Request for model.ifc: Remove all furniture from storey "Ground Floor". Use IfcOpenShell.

First a look at what the model holds.

```python
import ifcopenshell
import ifcopenshell.util.element

model = ifcopenshell.open("model.ifc")
print(model.schema)
storey = next(s for s in model.by_type("IfcBuildingStorey") if s.Name == "Ground Floor")
furniture = [e for e in ifcopenshell.util.element.get_decomposition(storey) if e.is_a("IfcFurnishingElement")]
seen = {}
for e in furniture:
    element_type = ifcopenshell.util.element.get_type(e)
    name = element_type.Name if element_type not in (None, e) else None
    seen[name] = seen.get(name, 0) + 1
for name, count in sorted(seen.items(), key=str):
    print(count, "x", name)
```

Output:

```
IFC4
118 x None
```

```python
import ifcopenshell
import ifcopenshell.api.root
import ifcopenshell.util.element

model = ifcopenshell.open("model.ifc")

storey = next(s for s in model.by_type("IfcBuildingStorey") if s.Name == "Ground Floor")
furniture = [e for e in ifcopenshell.util.element.get_decomposition(storey) if e.is_a("IfcFurnishingElement")]

for e in furniture:
    ifcopenshell.api.root.remove_product(model, product=e)
print(len(furniture), "removed")

model.write("model_edited.ifc")
```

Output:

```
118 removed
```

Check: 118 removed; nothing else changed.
